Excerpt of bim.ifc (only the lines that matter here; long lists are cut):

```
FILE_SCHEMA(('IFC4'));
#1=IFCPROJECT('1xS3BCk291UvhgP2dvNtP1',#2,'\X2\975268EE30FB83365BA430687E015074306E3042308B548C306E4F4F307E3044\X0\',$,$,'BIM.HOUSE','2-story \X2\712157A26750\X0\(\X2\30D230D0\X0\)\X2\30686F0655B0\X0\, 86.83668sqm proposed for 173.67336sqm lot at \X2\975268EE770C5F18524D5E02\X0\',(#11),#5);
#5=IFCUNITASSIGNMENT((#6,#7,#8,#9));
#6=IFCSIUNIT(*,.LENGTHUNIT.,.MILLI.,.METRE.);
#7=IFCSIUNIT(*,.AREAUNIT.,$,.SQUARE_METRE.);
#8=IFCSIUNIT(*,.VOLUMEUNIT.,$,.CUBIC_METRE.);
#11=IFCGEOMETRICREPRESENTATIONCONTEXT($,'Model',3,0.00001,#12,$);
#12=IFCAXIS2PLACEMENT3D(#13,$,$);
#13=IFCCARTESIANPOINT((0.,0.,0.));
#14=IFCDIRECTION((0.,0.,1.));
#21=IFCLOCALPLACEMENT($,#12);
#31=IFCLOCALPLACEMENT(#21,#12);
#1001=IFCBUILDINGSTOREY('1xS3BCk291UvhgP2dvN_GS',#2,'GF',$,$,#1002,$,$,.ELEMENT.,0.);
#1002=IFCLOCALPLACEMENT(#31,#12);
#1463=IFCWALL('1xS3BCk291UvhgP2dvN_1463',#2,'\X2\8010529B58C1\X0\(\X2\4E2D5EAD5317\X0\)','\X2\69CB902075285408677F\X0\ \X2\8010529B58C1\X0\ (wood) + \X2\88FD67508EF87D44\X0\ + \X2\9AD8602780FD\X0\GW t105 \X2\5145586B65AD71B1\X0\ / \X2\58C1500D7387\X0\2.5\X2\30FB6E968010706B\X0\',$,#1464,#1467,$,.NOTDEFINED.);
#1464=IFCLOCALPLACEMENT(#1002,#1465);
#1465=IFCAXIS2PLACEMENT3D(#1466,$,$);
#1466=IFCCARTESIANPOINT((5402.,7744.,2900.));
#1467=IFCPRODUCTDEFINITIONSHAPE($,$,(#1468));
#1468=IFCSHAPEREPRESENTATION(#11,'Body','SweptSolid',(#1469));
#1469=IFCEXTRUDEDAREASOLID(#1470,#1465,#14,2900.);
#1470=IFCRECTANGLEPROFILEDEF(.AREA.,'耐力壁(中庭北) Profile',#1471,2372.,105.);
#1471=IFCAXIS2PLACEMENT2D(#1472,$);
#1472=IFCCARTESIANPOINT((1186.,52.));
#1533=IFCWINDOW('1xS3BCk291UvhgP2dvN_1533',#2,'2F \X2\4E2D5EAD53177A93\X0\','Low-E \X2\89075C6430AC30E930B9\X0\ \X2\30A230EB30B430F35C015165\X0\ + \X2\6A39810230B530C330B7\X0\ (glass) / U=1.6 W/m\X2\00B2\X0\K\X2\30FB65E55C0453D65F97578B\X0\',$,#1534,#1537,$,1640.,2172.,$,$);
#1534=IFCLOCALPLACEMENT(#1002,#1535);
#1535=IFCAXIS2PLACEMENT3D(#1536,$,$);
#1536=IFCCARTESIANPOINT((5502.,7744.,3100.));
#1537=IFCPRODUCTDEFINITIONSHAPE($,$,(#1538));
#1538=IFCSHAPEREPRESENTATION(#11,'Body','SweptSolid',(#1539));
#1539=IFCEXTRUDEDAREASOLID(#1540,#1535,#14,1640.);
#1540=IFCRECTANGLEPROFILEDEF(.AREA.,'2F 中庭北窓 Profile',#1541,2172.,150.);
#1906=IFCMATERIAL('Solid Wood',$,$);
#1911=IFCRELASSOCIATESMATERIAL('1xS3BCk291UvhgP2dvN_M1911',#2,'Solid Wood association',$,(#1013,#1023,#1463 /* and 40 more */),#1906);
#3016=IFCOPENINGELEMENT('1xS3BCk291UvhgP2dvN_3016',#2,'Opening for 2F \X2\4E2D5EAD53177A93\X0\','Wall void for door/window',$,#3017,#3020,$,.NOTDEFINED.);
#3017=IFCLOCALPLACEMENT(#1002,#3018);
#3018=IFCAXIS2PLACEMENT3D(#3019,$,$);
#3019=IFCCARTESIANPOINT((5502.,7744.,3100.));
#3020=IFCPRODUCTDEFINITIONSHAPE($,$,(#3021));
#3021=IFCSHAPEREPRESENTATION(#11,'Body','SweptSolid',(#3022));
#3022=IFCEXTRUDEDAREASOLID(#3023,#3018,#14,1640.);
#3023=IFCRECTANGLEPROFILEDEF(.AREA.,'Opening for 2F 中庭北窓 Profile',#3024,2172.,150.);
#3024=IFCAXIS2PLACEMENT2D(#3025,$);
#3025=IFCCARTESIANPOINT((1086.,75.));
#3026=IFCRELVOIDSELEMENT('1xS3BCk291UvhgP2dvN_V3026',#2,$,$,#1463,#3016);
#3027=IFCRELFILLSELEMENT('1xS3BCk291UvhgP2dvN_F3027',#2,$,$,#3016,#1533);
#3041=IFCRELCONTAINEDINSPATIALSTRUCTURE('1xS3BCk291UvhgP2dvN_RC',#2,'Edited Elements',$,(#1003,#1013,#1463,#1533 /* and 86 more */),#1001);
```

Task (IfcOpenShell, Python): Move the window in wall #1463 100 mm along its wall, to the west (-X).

```python
import ifcopenshell
import ifcopenshell.api.geometry
import ifcopenshell.util.placement
import ifcopenshell.util.unit

model = ifcopenshell.open("bim.ifc")
unit_scale = ifcopenshell.util.unit.calculate_unit_scale(model)

window = model.by_id(1533)
opening = window.FillsVoids[0].RelatingOpeningElement
wall = opening.VoidsElements[0].RelatingBuildingElement

wall_matrix = ifcopenshell.util.placement.get_local_placement(wall.ObjectPlacement)
shift = wall_matrix[:3, 0] * -0.1 / unit_scale
before = ifcopenshell.util.placement.get_local_placement(window.ObjectPlacement)[:3, 3].copy()

# The window is not placed relative to its opening, so move both.
for product in (opening, window):
    matrix = ifcopenshell.util.placement.get_local_placement(product.ObjectPlacement)
    matrix[:3, 3] += shift
    ifcopenshell.api.geometry.edit_object_placement(model, product=product, matrix=matrix, is_si=False)

after = ifcopenshell.util.placement.get_local_placement(window.ObjectPlacement)[:3, 3]
print("window moved by", (after - before).round(3) + 0.0)

model.write("bim_edited.ifc")
```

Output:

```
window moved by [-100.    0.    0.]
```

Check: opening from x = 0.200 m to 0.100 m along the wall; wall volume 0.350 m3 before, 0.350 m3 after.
